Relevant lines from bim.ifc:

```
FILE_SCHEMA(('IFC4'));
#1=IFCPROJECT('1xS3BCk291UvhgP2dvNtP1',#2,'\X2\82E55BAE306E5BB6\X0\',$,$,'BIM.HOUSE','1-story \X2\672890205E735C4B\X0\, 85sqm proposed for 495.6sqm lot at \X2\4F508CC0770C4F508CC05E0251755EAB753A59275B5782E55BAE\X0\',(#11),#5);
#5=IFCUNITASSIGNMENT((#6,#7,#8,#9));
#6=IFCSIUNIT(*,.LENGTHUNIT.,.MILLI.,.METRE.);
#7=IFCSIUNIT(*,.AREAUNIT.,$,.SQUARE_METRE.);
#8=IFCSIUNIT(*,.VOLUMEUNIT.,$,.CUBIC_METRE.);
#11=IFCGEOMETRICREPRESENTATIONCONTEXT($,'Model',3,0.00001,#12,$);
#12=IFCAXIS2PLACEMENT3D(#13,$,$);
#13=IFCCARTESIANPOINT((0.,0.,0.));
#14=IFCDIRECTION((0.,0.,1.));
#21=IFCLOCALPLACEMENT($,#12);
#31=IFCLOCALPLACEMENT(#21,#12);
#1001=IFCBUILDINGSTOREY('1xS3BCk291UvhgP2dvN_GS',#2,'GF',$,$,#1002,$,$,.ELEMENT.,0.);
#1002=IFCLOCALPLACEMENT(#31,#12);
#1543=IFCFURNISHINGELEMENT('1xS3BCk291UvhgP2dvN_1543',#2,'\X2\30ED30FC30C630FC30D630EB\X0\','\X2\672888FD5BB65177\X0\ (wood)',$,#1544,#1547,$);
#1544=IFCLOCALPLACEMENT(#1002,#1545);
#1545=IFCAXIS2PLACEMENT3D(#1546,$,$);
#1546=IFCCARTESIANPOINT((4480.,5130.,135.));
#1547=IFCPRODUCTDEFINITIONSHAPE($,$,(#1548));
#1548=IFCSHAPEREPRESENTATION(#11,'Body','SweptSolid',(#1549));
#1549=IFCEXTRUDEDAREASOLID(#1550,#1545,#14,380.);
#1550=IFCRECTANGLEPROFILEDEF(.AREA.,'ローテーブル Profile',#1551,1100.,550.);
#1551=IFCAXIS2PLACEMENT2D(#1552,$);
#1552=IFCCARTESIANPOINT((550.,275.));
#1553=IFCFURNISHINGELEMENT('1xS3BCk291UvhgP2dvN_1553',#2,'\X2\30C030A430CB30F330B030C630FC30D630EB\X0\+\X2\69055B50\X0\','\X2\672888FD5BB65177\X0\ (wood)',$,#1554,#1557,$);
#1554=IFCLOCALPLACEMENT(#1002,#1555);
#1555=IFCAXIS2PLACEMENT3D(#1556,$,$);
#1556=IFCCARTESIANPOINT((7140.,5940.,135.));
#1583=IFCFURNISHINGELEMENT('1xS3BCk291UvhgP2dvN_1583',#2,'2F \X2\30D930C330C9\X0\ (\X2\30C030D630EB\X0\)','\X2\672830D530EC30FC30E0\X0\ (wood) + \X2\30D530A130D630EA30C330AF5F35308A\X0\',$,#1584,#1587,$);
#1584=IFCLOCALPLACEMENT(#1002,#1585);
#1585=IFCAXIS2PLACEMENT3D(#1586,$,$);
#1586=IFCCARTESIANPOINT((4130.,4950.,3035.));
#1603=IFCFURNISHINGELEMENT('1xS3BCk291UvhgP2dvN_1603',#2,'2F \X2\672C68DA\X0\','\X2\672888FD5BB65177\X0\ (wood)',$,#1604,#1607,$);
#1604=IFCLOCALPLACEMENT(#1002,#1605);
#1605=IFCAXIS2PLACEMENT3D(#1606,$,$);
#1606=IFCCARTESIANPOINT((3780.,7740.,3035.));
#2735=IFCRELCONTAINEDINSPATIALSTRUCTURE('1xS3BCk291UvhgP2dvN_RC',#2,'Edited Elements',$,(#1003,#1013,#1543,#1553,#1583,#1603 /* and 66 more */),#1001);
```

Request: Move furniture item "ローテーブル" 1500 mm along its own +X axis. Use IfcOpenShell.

```python
import ifcopenshell
import ifcopenshell.api.geometry
import ifcopenshell.util.placement

model = ifcopenshell.open("bim.ifc")

item = model.by_guid("1xS3BCk291UvhgP2dvN_1543")
matrix = ifcopenshell.util.placement.get_local_placement(item.ObjectPlacement)
matrix[:3, 3] += matrix[:3, 0] * 1500.0
ifcopenshell.api.geometry.edit_object_placement(model, product=item, matrix=matrix, is_si=False)

print(ifcopenshell.util.placement.get_local_placement(item.ObjectPlacement).round(3) + 0.0)

model.write("bim_rev.ifc")
```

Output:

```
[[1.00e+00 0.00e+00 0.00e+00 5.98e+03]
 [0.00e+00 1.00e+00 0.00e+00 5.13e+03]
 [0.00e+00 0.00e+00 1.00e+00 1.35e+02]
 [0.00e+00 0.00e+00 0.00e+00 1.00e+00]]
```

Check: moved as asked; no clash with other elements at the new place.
